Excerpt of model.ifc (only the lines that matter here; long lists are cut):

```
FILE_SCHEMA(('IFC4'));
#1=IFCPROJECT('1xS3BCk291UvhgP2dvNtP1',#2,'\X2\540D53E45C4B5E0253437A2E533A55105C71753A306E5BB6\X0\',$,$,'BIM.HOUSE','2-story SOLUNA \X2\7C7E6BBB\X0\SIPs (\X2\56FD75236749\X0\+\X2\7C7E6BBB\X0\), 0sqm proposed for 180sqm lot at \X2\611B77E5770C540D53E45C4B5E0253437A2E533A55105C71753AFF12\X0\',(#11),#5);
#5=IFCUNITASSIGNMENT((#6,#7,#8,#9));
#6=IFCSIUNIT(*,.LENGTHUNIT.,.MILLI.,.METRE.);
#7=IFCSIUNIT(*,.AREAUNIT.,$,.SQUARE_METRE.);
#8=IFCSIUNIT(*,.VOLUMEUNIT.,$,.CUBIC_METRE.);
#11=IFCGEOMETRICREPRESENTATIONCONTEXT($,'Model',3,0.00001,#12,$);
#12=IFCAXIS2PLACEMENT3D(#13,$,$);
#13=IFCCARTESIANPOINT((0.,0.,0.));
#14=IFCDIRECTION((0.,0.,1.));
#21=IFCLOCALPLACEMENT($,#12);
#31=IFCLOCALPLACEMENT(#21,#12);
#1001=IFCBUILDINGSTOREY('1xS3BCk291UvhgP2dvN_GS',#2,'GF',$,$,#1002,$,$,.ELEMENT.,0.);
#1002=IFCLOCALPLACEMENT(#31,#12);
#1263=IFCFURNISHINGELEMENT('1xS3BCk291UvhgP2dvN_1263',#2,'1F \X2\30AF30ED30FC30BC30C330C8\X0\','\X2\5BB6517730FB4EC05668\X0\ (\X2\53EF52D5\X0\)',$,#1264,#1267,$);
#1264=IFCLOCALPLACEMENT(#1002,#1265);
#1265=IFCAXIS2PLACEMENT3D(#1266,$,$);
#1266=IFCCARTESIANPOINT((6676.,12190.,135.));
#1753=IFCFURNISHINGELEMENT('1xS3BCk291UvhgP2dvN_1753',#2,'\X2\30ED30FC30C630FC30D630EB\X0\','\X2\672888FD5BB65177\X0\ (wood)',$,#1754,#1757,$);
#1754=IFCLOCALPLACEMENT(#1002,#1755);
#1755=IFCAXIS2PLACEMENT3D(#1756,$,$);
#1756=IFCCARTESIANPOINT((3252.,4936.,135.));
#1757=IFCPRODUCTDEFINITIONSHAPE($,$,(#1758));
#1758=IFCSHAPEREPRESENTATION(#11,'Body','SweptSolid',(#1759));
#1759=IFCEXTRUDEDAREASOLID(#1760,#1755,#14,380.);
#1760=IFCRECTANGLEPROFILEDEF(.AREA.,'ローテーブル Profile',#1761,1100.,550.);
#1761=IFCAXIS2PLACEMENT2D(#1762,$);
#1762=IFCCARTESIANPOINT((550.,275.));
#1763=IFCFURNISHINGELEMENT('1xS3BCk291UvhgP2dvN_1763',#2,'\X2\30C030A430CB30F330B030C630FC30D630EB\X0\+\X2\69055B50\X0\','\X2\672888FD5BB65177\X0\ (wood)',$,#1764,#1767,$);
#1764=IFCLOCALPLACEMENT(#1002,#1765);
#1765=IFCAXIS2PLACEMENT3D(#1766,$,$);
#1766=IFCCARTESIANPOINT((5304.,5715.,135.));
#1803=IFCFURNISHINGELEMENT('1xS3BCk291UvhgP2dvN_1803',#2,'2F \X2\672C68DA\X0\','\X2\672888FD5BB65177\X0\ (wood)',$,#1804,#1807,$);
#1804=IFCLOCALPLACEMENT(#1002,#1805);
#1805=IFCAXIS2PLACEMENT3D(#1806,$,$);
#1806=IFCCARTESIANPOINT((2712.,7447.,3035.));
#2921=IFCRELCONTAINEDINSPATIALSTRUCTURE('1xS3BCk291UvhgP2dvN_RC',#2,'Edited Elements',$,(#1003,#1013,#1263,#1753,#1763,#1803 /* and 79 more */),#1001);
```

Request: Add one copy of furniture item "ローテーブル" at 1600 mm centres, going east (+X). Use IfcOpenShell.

```python
import numpy as np
import ifcopenshell
import ifcopenshell.api.geometry
import ifcopenshell.api.root
import ifcopenshell.util.element
import ifcopenshell.util.placement

model = ifcopenshell.open("model.ifc")


def reuse_history(source, copy):
    """copy_class also copies each property set's owner history, people and application; keep the originals."""
    for rel in copy.IsDefinedBy:
        if rel.is_a("IfcRelDefinesByProperties") and (history := rel.RelatingPropertyDefinition.OwnerHistory):
            rel.RelatingPropertyDefinition.OwnerHistory = source.OwnerHistory
            ifcopenshell.util.element.remove_deep2(model, history)


source = model.by_id(1753)
base = ifcopenshell.util.placement.get_local_placement(source.ObjectPlacement)
step = np.array([1.0, 0.0, 0.0]) * 1600.0

for i in range(1, 2):
    copy = ifcopenshell.api.root.copy_class(model, product=source)
    copy.Representation = ifcopenshell.util.element.copy_deep(
        model, source.Representation, exclude=["IfcGeometricRepresentationContext", "IfcRepresentationMap"]
    )
    reuse_history(source, copy)
    matrix = base.copy()
    matrix[:3, 3] += i * step
    print("added at", matrix[:3, 3].round(3) + 0.0)
    ifcopenshell.api.geometry.edit_object_placement(model, product=copy, matrix=matrix, is_si=False)

model.write("model_updated.ifc")
```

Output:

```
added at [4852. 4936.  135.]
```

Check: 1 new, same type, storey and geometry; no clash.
